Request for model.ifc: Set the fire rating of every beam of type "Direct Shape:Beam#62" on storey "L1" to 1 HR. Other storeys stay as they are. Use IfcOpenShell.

First a look at what the model holds.

```python
import ifcopenshell
import ifcopenshell.util.element

model = ifcopenshell.open("model.ifc")
print(model.schema)
storey = next(s for s in model.by_type("IfcBuildingStorey") if s.Name == "L1")
beams = [e for e in ifcopenshell.util.element.get_decomposition(storey) if e.is_a("IfcBeam")]
seen = {}
for e in beams:
    element_type = ifcopenshell.util.element.get_type(e)
    key = (element_type.Name if element_type != e and element_type else None, ifcopenshell.util.element.get_pset(e, "Pset_BeamCommon", "FireRating"))
    seen[key] = seen.get(key, 0) + 1
for (name, value), count in sorted(seen.items(), key=str):
    print(count, "x", name, "|", value)
```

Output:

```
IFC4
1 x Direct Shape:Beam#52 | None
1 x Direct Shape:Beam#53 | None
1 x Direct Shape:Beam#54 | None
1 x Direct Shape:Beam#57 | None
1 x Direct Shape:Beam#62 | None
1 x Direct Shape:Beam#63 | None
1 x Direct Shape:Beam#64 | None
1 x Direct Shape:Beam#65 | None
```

```python
import ifcopenshell
import ifcopenshell.api.pset
import ifcopenshell.util.element

model = ifcopenshell.open("model.ifc")

storey = next(s for s in model.by_type("IfcBuildingStorey") if s.Name == "L1")
beams = [e for e in ifcopenshell.util.element.get_decomposition(storey) if e.is_a("IfcBeam")]

count = 0
for e in beams:
    element_type = ifcopenshell.util.element.get_type(e)
    if element_type in (None, e) or element_type.Name != "Direct Shape:Beam#62":
        continue
    # add_pset returns the element's existing set when there is one.
    pset = ifcopenshell.api.pset.add_pset(model, product=e, name="Pset_BeamCommon")
    ifcopenshell.api.pset.edit_pset(model, pset=pset, properties={"FireRating": "1 HR"})
    count += 1

print(count, "beams updated")

model.write("model-out.ifc")
```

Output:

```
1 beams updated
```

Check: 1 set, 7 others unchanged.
